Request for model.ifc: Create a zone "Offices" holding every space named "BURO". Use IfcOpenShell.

First a look at what the model holds.

```python
import ifcopenshell

model = ifcopenshell.open("model.ifc")
print(model.schema)
seen = {}
for space in model.by_type("IfcSpace"):
    seen[space.LongName] = seen.get(space.LongName, 0) + 1
for name, count in sorted(seen.items(), key=str):
    print(count, "x", name)
print("zones:", [z.Name for z in model.by_type("IfcZone")][:20])
```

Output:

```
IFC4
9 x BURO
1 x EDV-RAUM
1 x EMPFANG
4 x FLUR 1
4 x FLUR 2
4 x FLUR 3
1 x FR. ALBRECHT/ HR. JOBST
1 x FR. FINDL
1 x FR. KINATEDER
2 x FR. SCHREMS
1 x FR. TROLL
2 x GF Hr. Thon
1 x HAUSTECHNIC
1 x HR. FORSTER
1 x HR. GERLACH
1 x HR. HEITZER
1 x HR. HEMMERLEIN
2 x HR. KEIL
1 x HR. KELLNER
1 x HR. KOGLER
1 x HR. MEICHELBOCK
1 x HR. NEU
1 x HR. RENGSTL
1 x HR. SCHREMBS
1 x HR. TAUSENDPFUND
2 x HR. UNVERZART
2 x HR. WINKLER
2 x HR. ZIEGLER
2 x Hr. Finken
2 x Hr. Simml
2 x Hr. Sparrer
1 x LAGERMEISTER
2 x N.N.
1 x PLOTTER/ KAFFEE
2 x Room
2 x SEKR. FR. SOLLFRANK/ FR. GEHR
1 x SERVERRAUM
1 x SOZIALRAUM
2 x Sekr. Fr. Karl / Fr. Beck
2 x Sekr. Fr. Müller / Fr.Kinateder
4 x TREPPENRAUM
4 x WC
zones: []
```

```python
import ifcopenshell
import ifcopenshell.api.group
import ifcopenshell.api.root

model = ifcopenshell.open("model.ifc")

names = {"BURO"}
spaces = [s for s in model.by_type("IfcSpace") if s.LongName in names]

zone = ifcopenshell.api.root.create_entity(model, ifc_class="IfcZone", name="Offices")
ifcopenshell.api.group.assign_group(model, products=spaces, group=zone)
print(len(spaces), "spaces in", zone.Name)

model.write("model-out.ifc")
```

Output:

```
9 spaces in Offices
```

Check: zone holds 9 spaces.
